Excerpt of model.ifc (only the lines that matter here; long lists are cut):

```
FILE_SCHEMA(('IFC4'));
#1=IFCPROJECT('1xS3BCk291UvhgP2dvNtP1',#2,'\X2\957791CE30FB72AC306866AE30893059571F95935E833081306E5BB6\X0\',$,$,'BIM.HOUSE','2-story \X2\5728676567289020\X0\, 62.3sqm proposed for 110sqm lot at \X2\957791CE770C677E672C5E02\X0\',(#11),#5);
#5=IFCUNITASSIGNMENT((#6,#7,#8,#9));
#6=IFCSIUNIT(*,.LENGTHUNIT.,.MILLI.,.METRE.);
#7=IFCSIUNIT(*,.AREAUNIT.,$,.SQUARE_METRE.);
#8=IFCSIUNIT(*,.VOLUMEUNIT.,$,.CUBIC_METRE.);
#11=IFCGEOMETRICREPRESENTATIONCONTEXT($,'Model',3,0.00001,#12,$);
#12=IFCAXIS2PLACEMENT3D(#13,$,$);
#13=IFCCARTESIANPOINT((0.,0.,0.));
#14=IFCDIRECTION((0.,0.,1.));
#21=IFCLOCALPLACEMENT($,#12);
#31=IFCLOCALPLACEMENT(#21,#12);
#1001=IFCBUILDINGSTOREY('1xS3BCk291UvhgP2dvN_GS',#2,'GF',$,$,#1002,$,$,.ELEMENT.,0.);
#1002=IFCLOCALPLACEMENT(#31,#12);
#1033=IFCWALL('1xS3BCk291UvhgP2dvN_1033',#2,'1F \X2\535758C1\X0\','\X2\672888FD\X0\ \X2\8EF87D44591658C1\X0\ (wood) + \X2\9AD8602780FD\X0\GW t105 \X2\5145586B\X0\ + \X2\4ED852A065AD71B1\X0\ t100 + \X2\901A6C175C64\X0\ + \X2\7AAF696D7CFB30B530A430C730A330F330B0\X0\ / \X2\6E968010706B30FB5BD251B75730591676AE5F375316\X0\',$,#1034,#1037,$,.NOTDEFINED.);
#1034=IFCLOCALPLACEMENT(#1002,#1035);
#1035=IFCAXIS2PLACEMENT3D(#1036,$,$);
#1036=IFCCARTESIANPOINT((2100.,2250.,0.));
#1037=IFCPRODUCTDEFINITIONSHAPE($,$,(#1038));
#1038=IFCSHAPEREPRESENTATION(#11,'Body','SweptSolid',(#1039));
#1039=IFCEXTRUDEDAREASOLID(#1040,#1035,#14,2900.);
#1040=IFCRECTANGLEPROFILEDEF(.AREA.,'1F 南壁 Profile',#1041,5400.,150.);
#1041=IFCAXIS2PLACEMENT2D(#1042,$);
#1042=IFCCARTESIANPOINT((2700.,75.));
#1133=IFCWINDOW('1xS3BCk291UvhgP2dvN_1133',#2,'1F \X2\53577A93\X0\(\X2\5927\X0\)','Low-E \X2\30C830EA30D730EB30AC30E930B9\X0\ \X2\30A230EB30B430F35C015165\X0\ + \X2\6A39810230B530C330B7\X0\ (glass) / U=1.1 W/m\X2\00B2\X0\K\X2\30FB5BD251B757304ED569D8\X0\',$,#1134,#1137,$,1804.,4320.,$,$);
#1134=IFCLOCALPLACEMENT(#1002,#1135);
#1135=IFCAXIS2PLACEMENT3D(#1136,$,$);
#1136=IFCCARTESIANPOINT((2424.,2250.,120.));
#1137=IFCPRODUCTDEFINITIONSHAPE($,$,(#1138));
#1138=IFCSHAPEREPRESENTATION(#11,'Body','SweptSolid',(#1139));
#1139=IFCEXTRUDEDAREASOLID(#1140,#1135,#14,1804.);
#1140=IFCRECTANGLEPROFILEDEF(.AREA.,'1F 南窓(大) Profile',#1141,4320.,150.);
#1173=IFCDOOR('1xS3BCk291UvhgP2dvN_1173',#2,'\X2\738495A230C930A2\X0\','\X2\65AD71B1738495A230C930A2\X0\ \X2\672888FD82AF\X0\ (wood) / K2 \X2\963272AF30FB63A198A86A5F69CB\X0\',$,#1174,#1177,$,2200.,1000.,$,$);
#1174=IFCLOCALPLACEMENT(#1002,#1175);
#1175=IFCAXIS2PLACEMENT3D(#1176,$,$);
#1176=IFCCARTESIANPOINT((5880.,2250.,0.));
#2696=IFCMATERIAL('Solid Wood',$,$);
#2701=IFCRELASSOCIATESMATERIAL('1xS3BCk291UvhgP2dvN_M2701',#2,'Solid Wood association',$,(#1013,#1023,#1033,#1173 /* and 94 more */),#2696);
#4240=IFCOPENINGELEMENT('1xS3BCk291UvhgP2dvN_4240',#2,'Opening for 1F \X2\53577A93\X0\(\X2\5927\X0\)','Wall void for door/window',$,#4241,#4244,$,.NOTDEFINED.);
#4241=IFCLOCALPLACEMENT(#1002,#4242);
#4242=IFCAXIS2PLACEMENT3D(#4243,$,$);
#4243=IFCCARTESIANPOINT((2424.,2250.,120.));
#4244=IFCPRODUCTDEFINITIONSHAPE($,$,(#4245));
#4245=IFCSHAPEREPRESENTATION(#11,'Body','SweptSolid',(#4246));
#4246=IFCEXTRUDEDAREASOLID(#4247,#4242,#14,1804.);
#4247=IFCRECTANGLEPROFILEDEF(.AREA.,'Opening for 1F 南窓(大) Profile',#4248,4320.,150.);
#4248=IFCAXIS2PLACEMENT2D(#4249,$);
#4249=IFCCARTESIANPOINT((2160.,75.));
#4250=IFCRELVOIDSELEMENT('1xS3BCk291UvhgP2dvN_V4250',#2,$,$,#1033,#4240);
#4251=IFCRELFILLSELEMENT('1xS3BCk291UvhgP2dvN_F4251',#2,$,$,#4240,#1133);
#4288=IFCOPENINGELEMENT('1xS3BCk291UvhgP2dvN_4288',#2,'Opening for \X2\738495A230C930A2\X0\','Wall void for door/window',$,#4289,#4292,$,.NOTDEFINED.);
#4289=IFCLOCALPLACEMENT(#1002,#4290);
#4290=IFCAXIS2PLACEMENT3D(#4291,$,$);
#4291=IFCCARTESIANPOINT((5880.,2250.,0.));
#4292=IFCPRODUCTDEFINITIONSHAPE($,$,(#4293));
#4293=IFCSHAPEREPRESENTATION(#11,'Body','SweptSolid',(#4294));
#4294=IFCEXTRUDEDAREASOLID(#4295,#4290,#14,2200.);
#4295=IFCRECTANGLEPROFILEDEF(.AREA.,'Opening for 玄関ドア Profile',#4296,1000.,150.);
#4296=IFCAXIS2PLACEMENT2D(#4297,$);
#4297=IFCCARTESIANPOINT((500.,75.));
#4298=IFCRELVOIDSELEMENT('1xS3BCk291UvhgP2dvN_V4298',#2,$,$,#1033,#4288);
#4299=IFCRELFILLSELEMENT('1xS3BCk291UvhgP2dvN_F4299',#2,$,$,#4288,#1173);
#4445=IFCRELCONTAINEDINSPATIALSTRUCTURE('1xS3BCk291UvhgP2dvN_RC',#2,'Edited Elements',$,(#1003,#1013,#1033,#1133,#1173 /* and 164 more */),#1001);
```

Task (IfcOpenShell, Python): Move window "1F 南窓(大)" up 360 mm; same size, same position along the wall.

```python
import numpy as np
import ifcopenshell
import ifcopenshell.api.geometry
import ifcopenshell.util.placement
import ifcopenshell.util.unit

model = ifcopenshell.open("model.ifc")
unit_scale = ifcopenshell.util.unit.calculate_unit_scale(model)

window = model.by_guid("1xS3BCk291UvhgP2dvN_1133")
opening = window.FillsVoids[0].RelatingOpeningElement
dz = 0.36 / unit_scale

shift = np.array([0.0, 0.0, dz])
# The window is not placed relative to its opening, so move both.
for product in (opening, window):
    matrix = ifcopenshell.util.placement.get_local_placement(product.ObjectPlacement)
    matrix[:3, 3] += shift
    ifcopenshell.api.geometry.edit_object_placement(model, product=product, matrix=matrix, is_si=False)

print(f"moved by {dz * unit_scale:+.3f} m")

model.write("model_v2.ifc")
```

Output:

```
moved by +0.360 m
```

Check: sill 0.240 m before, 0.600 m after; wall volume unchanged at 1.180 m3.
